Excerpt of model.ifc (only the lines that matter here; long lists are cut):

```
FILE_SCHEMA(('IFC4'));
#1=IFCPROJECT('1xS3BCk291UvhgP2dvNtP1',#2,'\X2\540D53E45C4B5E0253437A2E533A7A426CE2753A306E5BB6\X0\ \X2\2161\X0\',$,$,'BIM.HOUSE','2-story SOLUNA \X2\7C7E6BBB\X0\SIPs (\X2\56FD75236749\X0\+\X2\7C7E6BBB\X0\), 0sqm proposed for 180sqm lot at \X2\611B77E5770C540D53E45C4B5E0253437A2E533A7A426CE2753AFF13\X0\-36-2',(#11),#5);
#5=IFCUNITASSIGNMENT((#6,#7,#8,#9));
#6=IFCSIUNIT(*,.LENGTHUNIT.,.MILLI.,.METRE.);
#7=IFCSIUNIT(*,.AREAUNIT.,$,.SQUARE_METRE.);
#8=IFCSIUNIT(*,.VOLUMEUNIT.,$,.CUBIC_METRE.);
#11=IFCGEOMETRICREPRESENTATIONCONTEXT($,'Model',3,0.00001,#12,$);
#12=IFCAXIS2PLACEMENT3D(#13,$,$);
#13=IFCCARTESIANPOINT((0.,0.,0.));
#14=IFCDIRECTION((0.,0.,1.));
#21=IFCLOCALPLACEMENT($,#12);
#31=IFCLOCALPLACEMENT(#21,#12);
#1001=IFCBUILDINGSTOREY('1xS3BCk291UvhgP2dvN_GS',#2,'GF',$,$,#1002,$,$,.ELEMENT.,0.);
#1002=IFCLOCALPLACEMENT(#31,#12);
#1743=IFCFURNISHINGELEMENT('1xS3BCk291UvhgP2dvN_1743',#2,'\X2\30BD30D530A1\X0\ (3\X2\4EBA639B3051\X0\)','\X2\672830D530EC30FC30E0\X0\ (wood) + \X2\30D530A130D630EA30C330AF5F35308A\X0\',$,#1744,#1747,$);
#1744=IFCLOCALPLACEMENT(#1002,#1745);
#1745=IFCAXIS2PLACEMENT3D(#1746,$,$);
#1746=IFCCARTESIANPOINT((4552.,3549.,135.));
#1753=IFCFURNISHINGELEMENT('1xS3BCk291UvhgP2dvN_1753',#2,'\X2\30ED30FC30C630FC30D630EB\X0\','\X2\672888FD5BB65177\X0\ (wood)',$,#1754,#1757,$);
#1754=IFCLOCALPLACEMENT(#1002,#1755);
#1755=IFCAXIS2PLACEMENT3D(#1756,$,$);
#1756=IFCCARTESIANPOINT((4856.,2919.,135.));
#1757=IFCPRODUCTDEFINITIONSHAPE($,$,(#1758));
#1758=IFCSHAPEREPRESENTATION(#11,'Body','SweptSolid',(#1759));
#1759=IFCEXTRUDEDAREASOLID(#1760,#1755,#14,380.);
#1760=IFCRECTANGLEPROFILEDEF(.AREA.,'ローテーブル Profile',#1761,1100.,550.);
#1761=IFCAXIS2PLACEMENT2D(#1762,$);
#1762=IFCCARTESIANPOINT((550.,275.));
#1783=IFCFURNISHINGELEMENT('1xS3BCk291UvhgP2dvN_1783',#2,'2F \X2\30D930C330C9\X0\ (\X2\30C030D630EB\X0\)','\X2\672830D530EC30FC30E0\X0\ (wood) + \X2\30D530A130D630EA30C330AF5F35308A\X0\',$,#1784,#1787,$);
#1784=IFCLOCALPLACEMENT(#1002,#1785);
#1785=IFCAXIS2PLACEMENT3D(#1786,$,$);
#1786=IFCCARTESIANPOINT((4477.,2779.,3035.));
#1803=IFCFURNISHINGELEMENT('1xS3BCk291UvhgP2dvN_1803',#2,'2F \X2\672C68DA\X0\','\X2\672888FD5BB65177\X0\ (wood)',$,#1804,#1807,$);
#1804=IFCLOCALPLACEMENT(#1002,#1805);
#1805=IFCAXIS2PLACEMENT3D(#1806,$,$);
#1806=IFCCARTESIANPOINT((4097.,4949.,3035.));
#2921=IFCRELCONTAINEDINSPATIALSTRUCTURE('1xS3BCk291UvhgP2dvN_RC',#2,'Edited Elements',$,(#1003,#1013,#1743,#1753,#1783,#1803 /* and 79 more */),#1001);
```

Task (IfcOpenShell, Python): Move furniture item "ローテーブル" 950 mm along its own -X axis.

```python
import ifcopenshell
import ifcopenshell.api.geometry
import ifcopenshell.util.placement
import ifcopenshell.util.unit

model = ifcopenshell.open("model.ifc")
unit_scale = ifcopenshell.util.unit.calculate_unit_scale(model)

item = model.by_guid("1xS3BCk291UvhgP2dvN_1753")
matrix = ifcopenshell.util.placement.get_local_placement(item.ObjectPlacement)
matrix[:3, 3] -= matrix[:3, 0] * 0.95 / unit_scale
ifcopenshell.api.geometry.edit_object_placement(model, product=item, matrix=matrix, is_si=False)

print(ifcopenshell.util.placement.get_local_placement(item.ObjectPlacement).round(3) + 0.0)

model.write("model_edited.ifc")
```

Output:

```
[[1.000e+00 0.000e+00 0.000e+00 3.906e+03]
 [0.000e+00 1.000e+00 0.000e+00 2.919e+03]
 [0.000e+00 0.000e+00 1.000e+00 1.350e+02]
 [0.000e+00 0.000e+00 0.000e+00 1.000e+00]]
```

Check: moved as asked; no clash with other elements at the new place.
